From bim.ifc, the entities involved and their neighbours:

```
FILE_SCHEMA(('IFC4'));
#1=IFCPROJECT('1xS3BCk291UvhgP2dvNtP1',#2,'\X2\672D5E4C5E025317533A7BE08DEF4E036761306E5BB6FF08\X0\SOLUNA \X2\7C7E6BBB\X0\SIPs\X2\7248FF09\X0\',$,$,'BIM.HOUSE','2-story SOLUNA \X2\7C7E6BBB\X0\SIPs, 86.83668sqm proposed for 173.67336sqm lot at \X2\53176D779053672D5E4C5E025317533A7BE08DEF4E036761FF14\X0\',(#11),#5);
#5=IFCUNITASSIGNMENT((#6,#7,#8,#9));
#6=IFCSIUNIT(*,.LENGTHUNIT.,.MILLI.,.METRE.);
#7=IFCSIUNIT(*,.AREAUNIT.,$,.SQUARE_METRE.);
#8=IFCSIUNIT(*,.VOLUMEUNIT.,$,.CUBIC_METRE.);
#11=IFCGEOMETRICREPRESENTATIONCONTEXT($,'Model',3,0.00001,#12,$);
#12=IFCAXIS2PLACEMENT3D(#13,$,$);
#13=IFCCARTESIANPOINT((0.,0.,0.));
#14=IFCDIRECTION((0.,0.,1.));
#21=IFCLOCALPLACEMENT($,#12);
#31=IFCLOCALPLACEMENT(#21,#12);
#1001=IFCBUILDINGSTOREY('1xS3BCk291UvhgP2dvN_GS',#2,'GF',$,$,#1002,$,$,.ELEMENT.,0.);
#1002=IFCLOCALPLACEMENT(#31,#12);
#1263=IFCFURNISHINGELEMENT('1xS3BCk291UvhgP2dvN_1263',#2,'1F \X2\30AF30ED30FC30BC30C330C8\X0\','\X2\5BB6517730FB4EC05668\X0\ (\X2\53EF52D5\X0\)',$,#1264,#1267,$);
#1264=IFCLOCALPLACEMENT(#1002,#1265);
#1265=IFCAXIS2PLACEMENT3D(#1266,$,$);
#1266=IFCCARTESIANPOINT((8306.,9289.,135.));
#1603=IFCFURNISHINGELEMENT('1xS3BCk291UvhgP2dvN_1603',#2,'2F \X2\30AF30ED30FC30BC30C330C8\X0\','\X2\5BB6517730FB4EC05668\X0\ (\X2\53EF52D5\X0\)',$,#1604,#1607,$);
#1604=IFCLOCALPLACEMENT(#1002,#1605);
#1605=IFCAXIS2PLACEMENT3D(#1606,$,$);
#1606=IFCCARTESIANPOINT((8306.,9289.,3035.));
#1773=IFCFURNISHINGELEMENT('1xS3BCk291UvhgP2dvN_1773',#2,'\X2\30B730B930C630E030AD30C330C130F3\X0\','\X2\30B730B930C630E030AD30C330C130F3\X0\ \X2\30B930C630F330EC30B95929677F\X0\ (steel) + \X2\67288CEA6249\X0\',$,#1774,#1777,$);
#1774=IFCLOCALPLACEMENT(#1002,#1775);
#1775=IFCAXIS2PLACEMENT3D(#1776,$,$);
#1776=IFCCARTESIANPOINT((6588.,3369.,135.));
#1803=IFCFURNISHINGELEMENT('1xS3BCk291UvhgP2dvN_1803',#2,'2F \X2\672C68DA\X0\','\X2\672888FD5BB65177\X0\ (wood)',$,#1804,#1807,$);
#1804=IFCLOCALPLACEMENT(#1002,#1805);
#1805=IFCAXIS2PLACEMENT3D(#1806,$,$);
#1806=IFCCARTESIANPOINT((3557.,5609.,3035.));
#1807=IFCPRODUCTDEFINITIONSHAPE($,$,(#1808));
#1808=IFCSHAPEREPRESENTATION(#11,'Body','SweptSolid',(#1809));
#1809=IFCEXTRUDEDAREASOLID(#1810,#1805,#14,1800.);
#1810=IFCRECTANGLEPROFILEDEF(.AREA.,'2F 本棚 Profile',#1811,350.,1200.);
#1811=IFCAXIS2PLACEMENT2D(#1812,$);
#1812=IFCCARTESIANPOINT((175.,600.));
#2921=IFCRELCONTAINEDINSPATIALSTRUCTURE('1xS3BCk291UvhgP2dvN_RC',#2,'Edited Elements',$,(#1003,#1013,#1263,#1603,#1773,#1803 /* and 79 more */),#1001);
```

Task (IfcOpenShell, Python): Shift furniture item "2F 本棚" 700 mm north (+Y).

```python
import ifcopenshell
import ifcopenshell.api.geometry
import ifcopenshell.util.placement

model = ifcopenshell.open("bim.ifc")

item = model.by_guid("1xS3BCk291UvhgP2dvN_1803")
matrix = ifcopenshell.util.placement.get_local_placement(item.ObjectPlacement)
matrix[1, 3] += 700.0
ifcopenshell.api.geometry.edit_object_placement(model, product=item, matrix=matrix, is_si=False)

print(ifcopenshell.util.placement.get_local_placement(item.ObjectPlacement).round(3) + 0.0)

model.write("bim_edited.ifc")
```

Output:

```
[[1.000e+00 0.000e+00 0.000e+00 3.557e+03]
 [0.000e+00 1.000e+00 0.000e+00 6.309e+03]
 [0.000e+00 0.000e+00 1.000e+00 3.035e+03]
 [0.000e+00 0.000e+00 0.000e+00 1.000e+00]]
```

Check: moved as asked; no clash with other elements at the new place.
